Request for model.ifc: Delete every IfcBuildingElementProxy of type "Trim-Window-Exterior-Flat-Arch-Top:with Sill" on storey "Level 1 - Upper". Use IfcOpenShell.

First a look at what the model holds.

```python
import ifcopenshell
import ifcopenshell.util.element

model = ifcopenshell.open("model.ifc")
print(model.schema)
storey = next(s for s in model.by_type("IfcBuildingStorey") if s.Name == "Level 1 - Upper")
proxies = [e for e in ifcopenshell.util.element.get_decomposition(storey) if e.is_a("IfcBuildingElementProxy")]
seen = {}
for e in proxies:
    element_type = ifcopenshell.util.element.get_type(e)
    name = element_type.Name if element_type not in (None, e) else None
    seen[name] = seen.get(name, 0) + 1
for name, count in sorted(seen.items(), key=str):
    print(count, "x", name)
```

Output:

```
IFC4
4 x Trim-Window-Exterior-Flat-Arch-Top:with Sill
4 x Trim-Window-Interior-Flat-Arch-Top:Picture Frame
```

```python
import ifcopenshell
import ifcopenshell.api.root
import ifcopenshell.util.element

model = ifcopenshell.open("model.ifc")

storey = next(s for s in model.by_type("IfcBuildingStorey") if s.Name == "Level 1 - Upper")
proxies = [e for e in ifcopenshell.util.element.get_decomposition(storey) if e.is_a("IfcBuildingElementProxy")]
targets = [e for e in proxies if (t := ifcopenshell.util.element.get_type(e)) not in (None, e) and t.Name == "Trim-Window-Exterior-Flat-Arch-Top:with Sill"]

for e in targets:
    ifcopenshell.api.root.remove_product(model, product=e)
print(len(targets), "removed")

model.write("model_edited.ifc")
```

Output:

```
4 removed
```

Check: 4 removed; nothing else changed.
